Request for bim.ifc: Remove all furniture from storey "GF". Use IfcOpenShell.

First a look at what the model holds.

```python
import ifcopenshell
import ifcopenshell.util.element

model = ifcopenshell.open("bim.ifc")
print(model.schema)
storey = next(s for s in model.by_type("IfcBuildingStorey") if s.Name == "GF")
furniture = [e for e in ifcopenshell.util.element.get_decomposition(storey) if e.is_a("IfcFurnishingElement")]
seen = {}
for e in furniture:
    element_type = ifcopenshell.util.element.get_type(e)
    name = element_type.Name if element_type not in (None, e) else None
    seen[name] = seen.get(name, 0) + 1
for name, count in sorted(seen.items(), key=str):
    print(count, "x", name)
```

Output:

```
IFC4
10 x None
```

```python
import ifcopenshell
import ifcopenshell.api.root
import ifcopenshell.util.element

model = ifcopenshell.open("bim.ifc")

storey = next(s for s in model.by_type("IfcBuildingStorey") if s.Name == "GF")
furniture = [e for e in ifcopenshell.util.element.get_decomposition(storey) if e.is_a("IfcFurnishingElement")]

for e in furniture:
    ifcopenshell.api.root.remove_product(model, product=e)
print(len(furniture), "removed")

model.write("bim_edited.ifc")
```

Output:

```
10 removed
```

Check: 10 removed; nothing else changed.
